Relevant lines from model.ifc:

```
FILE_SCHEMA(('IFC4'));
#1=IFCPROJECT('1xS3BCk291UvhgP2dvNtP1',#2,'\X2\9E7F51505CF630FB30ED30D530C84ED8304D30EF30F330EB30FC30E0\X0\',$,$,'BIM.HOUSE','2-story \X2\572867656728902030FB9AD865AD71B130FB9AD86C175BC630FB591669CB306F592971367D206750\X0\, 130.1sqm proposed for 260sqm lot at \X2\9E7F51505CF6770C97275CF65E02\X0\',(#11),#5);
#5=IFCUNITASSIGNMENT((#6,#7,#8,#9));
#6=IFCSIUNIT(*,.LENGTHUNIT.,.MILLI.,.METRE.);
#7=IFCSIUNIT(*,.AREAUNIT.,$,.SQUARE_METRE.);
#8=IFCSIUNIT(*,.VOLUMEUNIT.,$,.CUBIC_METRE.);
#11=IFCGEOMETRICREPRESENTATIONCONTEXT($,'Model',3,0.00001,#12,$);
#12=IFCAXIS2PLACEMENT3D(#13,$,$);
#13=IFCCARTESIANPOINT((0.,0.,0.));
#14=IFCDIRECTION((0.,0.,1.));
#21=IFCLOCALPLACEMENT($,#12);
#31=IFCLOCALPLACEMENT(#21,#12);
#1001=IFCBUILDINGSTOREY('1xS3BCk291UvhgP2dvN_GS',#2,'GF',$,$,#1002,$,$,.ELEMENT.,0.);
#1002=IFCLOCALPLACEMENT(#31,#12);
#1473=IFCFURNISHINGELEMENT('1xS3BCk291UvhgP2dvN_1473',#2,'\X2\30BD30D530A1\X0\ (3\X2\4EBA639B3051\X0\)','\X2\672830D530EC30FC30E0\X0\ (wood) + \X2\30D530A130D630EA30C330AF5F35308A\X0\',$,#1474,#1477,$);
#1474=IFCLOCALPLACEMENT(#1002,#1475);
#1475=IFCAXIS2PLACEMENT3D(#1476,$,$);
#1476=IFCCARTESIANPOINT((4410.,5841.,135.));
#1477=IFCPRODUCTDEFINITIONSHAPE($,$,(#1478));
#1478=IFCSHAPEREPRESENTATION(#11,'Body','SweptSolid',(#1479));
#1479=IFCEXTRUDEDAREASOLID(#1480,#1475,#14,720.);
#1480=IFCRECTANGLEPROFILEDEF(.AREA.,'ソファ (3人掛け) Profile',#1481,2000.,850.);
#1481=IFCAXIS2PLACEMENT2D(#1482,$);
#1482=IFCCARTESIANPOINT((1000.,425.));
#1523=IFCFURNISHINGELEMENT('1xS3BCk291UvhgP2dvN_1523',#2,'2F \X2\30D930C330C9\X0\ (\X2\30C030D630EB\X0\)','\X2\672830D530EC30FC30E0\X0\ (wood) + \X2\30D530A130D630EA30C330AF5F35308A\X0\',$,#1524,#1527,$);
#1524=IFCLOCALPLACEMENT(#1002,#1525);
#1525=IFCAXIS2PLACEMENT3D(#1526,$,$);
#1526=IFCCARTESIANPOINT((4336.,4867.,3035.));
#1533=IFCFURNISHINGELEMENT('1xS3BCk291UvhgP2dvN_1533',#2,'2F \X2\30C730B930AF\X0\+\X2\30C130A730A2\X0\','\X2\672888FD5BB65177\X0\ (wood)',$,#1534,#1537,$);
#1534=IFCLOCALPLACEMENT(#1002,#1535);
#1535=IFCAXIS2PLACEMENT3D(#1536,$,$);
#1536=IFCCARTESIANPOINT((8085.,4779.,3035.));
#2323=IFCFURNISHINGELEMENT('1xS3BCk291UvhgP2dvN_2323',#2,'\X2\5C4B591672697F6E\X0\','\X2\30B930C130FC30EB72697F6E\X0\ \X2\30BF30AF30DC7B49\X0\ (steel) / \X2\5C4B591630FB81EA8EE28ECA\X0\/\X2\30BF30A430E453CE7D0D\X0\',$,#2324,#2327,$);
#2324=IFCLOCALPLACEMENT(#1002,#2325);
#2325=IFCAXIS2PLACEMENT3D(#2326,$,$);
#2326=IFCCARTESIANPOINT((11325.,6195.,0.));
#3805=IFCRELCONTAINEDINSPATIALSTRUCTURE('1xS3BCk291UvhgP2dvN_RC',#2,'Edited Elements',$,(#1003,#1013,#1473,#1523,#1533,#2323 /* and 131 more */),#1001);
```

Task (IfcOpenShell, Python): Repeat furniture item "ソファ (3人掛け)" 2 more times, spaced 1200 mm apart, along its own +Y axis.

```python
import ifcopenshell
import ifcopenshell.api.geometry
import ifcopenshell.api.root
import ifcopenshell.util.element
import ifcopenshell.util.placement

model = ifcopenshell.open("model.ifc")


def reuse_history(source, copy):
    """copy_class also copies each property set's owner history, people and application; keep the originals."""
    for rel in copy.IsDefinedBy:
        if rel.is_a("IfcRelDefinesByProperties") and (history := rel.RelatingPropertyDefinition.OwnerHistory):
            rel.RelatingPropertyDefinition.OwnerHistory = source.OwnerHistory
            ifcopenshell.util.element.remove_deep2(model, history)


source = model.by_id(1473)
base = ifcopenshell.util.placement.get_local_placement(source.ObjectPlacement)
step = base[:3, 1] * 1200.0

for i in range(1, 3):
    copy = ifcopenshell.api.root.copy_class(model, product=source)
    copy.Representation = ifcopenshell.util.element.copy_deep(
        model, source.Representation, exclude=["IfcGeometricRepresentationContext", "IfcRepresentationMap"]
    )
    reuse_history(source, copy)
    matrix = base.copy()
    matrix[:3, 3] += i * step
    print("added at", matrix[:3, 3].round(3) + 0.0)
    ifcopenshell.api.geometry.edit_object_placement(model, product=copy, matrix=matrix, is_si=False)

model.write("model_edited.ifc")
```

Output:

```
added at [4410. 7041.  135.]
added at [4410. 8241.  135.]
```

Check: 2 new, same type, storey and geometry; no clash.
